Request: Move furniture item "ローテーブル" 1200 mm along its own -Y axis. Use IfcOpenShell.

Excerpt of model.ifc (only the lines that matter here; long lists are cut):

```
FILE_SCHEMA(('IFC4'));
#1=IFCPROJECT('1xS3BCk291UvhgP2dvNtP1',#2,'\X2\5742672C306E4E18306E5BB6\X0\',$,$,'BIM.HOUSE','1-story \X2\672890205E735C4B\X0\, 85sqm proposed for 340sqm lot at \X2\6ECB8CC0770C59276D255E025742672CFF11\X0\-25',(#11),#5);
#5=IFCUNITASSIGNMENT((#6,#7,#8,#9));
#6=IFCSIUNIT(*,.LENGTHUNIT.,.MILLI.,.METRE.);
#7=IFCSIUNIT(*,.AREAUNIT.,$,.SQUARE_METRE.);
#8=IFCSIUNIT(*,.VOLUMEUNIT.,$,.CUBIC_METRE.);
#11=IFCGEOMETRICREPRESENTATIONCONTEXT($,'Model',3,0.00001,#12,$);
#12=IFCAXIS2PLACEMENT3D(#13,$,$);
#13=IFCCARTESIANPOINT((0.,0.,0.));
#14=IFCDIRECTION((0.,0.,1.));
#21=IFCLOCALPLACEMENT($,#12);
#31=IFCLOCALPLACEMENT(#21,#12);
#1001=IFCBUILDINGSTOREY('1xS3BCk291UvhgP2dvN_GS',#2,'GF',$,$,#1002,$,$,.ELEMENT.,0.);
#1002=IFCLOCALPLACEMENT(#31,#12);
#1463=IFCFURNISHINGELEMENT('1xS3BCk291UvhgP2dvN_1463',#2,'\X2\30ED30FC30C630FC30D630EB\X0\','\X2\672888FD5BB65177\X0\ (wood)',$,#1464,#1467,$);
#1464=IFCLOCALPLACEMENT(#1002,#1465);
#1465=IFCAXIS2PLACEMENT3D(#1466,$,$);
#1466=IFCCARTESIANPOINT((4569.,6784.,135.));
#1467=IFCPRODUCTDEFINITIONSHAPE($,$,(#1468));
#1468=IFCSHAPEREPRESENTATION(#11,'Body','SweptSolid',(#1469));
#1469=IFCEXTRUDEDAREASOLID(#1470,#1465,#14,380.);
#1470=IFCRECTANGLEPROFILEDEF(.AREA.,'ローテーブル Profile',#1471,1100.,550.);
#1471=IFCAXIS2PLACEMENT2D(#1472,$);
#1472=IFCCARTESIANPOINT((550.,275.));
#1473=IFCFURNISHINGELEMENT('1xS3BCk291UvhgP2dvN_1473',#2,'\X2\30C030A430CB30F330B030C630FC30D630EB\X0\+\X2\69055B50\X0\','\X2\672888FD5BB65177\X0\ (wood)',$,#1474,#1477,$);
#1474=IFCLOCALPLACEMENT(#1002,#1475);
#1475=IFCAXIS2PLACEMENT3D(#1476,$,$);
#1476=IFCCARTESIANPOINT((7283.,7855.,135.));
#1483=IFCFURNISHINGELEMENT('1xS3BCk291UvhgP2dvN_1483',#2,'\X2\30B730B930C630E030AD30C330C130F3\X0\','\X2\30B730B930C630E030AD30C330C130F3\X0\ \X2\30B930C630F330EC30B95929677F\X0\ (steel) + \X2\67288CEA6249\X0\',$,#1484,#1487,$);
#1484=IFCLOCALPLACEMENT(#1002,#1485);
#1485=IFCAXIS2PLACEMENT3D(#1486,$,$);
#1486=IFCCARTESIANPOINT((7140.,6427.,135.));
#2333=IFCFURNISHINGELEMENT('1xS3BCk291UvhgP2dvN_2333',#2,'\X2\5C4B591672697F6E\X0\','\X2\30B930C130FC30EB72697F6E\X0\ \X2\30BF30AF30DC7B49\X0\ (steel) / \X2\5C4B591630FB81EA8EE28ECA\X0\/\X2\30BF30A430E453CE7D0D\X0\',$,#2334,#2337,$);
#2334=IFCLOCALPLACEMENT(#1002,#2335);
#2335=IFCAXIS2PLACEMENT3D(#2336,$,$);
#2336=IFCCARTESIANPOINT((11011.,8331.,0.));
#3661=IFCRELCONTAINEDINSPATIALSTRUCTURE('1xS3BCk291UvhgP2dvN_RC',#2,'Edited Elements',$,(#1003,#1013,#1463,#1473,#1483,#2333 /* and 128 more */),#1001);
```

```python
import ifcopenshell
import ifcopenshell.api.geometry
import ifcopenshell.util.placement
import ifcopenshell.util.unit

model = ifcopenshell.open("model.ifc")
unit_scale = ifcopenshell.util.unit.calculate_unit_scale(model)

item = model.by_id(1463)
matrix = ifcopenshell.util.placement.get_local_placement(item.ObjectPlacement)
matrix[:3, 3] -= matrix[:3, 1] * 1.2 / unit_scale
ifcopenshell.api.geometry.edit_object_placement(model, product=item, matrix=matrix, is_si=False)

print(ifcopenshell.util.placement.get_local_placement(item.ObjectPlacement).round(3) + 0.0)

model.write("model_updated.ifc")
```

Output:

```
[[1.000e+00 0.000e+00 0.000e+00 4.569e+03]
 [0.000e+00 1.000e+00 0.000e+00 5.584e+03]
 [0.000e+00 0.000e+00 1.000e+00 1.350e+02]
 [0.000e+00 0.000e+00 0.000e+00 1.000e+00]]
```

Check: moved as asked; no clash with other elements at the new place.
